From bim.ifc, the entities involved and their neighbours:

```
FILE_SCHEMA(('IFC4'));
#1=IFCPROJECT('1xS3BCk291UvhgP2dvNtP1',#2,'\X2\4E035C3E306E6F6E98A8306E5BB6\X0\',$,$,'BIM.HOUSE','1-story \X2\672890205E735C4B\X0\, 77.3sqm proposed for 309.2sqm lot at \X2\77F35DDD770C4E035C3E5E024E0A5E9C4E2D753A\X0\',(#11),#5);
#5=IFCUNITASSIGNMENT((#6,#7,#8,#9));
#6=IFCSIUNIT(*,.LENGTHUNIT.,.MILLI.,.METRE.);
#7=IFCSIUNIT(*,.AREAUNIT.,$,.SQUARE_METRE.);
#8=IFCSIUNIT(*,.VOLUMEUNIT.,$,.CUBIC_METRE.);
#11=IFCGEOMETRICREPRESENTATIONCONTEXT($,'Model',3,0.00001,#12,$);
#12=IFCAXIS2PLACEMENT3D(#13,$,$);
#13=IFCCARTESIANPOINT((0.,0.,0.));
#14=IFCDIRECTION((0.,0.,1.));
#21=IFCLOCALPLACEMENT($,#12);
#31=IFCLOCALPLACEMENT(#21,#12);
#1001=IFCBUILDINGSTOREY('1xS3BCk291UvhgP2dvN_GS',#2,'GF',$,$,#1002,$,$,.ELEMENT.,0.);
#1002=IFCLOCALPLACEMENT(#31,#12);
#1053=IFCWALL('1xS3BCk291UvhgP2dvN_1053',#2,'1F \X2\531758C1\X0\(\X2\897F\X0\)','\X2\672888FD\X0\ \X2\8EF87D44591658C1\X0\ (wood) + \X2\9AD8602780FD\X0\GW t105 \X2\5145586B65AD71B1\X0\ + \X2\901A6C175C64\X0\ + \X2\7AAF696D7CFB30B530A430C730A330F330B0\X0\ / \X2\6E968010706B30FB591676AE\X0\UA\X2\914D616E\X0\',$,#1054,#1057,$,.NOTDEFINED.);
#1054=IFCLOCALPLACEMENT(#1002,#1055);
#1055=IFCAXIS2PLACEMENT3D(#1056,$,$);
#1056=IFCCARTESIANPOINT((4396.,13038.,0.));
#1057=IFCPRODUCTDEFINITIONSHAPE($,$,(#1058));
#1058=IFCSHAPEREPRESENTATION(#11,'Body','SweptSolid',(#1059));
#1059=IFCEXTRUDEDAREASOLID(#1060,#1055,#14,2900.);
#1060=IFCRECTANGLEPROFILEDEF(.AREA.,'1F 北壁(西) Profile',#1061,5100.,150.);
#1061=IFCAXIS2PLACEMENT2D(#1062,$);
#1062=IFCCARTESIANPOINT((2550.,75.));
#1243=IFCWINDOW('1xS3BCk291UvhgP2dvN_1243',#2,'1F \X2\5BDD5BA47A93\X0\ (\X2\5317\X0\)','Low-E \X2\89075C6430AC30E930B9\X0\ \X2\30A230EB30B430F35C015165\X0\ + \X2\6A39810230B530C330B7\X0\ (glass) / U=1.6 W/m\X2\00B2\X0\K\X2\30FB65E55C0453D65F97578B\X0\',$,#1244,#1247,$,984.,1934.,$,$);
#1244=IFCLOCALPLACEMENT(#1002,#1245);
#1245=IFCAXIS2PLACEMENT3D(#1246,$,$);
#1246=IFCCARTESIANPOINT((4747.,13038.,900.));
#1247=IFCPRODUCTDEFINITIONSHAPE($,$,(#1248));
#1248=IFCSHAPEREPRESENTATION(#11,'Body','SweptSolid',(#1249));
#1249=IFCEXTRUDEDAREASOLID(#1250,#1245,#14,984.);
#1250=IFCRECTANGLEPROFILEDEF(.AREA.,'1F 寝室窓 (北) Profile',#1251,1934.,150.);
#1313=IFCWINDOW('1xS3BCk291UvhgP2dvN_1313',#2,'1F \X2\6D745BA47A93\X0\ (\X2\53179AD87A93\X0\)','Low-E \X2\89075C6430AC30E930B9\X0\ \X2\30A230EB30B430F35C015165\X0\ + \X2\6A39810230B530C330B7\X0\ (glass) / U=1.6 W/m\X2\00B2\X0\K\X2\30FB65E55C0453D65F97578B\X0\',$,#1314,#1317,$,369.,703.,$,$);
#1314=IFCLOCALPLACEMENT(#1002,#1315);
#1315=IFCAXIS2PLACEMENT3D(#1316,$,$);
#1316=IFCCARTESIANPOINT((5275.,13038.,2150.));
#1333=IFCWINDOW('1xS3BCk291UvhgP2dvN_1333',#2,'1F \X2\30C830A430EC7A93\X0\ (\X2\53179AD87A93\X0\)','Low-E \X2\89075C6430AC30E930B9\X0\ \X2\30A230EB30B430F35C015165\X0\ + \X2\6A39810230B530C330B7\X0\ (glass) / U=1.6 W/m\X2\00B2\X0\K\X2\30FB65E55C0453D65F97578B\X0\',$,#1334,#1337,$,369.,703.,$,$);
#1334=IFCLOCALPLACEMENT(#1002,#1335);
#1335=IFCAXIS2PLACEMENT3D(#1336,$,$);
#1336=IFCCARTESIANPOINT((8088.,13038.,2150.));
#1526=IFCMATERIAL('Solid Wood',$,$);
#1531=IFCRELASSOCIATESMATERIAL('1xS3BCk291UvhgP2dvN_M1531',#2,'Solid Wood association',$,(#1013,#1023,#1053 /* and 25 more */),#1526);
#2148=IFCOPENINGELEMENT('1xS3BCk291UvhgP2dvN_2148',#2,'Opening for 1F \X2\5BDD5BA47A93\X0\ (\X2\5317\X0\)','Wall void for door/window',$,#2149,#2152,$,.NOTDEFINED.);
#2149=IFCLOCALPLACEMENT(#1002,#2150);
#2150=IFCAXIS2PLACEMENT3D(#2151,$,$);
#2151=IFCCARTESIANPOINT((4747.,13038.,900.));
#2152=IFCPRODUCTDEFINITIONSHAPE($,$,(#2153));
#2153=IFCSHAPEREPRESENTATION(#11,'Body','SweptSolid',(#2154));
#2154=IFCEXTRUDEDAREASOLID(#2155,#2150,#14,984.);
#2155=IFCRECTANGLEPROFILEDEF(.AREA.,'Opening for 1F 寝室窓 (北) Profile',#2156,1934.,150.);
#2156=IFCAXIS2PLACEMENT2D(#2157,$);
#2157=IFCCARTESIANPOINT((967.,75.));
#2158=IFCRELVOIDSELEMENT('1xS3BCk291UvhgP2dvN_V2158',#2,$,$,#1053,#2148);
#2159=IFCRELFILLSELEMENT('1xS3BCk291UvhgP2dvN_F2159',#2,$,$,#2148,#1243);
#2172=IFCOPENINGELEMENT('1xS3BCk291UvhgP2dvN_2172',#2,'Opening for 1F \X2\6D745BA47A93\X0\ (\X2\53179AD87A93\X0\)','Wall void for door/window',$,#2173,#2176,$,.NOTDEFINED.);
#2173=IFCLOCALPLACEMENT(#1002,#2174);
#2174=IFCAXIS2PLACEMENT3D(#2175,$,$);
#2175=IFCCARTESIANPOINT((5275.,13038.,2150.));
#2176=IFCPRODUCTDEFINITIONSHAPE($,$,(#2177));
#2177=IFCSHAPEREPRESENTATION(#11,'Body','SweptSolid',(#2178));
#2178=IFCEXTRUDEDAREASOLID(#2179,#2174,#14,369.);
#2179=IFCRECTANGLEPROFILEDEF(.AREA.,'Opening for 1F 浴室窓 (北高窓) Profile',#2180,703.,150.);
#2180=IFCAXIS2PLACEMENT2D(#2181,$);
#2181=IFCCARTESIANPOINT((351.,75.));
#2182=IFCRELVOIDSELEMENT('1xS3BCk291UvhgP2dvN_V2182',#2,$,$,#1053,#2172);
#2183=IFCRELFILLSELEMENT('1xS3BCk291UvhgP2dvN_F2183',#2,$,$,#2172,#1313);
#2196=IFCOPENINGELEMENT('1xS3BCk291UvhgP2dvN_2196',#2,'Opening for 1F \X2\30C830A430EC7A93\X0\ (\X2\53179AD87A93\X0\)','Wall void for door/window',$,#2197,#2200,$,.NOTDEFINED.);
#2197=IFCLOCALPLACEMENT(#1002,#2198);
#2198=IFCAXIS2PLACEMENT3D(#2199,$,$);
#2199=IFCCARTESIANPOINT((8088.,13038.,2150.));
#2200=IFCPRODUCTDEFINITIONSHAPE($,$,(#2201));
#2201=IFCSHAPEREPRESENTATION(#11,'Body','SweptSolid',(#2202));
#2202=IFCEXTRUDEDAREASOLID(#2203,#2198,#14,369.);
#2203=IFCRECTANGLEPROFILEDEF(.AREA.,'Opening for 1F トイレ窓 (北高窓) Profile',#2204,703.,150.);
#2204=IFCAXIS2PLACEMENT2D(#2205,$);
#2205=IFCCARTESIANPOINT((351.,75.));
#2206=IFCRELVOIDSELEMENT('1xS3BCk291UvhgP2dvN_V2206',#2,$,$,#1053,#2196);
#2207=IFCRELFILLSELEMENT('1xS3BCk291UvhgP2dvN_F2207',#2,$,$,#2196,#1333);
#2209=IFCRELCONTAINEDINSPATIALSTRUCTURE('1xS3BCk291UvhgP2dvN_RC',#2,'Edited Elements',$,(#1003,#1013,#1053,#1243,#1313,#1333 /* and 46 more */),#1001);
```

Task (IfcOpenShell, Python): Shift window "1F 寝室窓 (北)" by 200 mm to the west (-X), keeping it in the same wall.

```python
import ifcopenshell
import ifcopenshell.api.geometry
import ifcopenshell.util.placement
import ifcopenshell.util.unit

model = ifcopenshell.open("bim.ifc")
unit_scale = ifcopenshell.util.unit.calculate_unit_scale(model)

window = model.by_id(1243)
opening = window.FillsVoids[0].RelatingOpeningElement
wall = opening.VoidsElements[0].RelatingBuildingElement

wall_matrix = ifcopenshell.util.placement.get_local_placement(wall.ObjectPlacement)
shift = wall_matrix[:3, 0] * -0.2 / unit_scale
before = ifcopenshell.util.placement.get_local_placement(window.ObjectPlacement)[:3, 3].copy()

# The window is not placed relative to its opening, so move both.
for product in (opening, window):
    matrix = ifcopenshell.util.placement.get_local_placement(product.ObjectPlacement)
    matrix[:3, 3] += shift
    ifcopenshell.api.geometry.edit_object_placement(model, product=product, matrix=matrix, is_si=False)

after = ifcopenshell.util.placement.get_local_placement(window.ObjectPlacement)[:3, 3]
print("window moved by", (after - before).round(3) + 0.0)

model.write("bim_rev.ifc")
```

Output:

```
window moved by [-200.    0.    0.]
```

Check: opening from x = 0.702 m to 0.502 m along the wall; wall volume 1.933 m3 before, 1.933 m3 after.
